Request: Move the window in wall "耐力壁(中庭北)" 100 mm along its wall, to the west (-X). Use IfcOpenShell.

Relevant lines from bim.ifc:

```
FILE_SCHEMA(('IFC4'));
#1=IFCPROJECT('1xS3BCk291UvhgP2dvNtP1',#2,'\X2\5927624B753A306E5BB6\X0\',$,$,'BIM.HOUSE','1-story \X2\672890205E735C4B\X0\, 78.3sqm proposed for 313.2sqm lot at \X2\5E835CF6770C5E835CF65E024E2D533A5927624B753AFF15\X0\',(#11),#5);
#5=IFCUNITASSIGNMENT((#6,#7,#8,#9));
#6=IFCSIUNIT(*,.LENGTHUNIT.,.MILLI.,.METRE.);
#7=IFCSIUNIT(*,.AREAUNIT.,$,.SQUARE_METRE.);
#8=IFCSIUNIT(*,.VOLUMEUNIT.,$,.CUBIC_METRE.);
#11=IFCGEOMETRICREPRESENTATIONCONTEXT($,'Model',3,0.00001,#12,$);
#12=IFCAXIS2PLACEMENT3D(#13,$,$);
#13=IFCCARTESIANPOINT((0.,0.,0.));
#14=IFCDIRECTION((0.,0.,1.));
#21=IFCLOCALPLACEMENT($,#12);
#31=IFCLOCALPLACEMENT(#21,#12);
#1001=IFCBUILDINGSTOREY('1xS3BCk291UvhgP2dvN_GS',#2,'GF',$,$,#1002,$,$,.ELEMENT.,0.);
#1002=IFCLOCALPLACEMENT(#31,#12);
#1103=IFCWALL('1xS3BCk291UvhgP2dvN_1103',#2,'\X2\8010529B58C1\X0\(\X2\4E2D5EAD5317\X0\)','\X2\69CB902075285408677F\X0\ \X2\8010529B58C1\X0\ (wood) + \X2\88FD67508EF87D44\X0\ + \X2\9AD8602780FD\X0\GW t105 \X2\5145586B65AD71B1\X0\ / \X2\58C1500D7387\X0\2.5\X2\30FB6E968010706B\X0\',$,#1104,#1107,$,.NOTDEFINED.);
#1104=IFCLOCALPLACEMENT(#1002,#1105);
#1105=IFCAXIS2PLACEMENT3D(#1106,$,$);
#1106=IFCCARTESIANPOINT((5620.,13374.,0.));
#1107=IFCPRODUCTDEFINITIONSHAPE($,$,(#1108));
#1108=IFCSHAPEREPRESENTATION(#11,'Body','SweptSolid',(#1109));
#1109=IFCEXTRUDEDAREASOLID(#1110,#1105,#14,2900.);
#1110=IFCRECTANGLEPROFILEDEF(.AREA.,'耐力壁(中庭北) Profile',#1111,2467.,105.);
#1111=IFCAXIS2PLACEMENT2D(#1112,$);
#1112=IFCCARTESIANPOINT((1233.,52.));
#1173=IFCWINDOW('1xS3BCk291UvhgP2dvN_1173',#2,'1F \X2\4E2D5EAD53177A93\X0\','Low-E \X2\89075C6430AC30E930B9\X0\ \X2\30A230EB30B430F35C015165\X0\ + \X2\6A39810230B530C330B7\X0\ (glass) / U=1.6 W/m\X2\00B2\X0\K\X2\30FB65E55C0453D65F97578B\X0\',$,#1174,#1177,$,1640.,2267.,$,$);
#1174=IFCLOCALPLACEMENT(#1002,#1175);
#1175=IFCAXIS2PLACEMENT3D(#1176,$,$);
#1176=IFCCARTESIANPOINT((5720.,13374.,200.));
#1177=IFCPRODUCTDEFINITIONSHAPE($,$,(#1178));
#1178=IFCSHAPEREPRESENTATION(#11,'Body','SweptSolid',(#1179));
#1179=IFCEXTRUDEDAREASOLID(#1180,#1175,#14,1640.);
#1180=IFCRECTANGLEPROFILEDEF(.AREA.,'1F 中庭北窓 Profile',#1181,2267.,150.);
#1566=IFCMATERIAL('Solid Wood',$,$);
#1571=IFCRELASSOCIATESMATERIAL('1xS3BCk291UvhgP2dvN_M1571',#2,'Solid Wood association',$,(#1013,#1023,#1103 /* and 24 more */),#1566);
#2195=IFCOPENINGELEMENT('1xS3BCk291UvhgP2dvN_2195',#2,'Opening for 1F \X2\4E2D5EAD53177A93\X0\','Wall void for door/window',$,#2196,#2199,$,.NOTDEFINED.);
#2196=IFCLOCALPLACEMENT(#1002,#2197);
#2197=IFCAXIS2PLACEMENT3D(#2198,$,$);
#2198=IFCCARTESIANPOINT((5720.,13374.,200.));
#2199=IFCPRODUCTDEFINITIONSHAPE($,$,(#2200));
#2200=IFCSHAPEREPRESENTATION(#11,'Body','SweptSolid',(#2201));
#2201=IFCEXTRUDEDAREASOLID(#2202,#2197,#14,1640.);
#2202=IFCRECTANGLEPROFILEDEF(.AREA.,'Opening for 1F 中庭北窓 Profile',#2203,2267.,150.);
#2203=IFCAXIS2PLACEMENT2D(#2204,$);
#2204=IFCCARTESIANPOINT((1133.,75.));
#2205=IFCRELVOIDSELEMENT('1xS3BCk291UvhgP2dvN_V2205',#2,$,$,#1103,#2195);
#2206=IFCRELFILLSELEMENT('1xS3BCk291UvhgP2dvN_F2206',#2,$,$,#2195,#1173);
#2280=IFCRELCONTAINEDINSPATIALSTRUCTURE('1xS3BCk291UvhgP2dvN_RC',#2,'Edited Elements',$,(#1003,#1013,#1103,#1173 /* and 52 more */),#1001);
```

```python
import ifcopenshell
import ifcopenshell.api.geometry
import ifcopenshell.util.placement

model = ifcopenshell.open("bim.ifc")

window = model.by_id(1173)
opening = window.FillsVoids[0].RelatingOpeningElement
wall = opening.VoidsElements[0].RelatingBuildingElement

wall_matrix = ifcopenshell.util.placement.get_local_placement(wall.ObjectPlacement)
shift = wall_matrix[:3, 0] * -100.0
before = ifcopenshell.util.placement.get_local_placement(window.ObjectPlacement)[:3, 3].copy()

# The window is not placed relative to its opening, so move both.
for product in (opening, window):
    matrix = ifcopenshell.util.placement.get_local_placement(product.ObjectPlacement)
    matrix[:3, 3] += shift
    ifcopenshell.api.geometry.edit_object_placement(model, product=product, matrix=matrix, is_si=False)

after = ifcopenshell.util.placement.get_local_placement(window.ObjectPlacement)[:3, 3]
print("window moved by", (after - before).round(3) + 0.0)

model.write("bim_updated.ifc")
```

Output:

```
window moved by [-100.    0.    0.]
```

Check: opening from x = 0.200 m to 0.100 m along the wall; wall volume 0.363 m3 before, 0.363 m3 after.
